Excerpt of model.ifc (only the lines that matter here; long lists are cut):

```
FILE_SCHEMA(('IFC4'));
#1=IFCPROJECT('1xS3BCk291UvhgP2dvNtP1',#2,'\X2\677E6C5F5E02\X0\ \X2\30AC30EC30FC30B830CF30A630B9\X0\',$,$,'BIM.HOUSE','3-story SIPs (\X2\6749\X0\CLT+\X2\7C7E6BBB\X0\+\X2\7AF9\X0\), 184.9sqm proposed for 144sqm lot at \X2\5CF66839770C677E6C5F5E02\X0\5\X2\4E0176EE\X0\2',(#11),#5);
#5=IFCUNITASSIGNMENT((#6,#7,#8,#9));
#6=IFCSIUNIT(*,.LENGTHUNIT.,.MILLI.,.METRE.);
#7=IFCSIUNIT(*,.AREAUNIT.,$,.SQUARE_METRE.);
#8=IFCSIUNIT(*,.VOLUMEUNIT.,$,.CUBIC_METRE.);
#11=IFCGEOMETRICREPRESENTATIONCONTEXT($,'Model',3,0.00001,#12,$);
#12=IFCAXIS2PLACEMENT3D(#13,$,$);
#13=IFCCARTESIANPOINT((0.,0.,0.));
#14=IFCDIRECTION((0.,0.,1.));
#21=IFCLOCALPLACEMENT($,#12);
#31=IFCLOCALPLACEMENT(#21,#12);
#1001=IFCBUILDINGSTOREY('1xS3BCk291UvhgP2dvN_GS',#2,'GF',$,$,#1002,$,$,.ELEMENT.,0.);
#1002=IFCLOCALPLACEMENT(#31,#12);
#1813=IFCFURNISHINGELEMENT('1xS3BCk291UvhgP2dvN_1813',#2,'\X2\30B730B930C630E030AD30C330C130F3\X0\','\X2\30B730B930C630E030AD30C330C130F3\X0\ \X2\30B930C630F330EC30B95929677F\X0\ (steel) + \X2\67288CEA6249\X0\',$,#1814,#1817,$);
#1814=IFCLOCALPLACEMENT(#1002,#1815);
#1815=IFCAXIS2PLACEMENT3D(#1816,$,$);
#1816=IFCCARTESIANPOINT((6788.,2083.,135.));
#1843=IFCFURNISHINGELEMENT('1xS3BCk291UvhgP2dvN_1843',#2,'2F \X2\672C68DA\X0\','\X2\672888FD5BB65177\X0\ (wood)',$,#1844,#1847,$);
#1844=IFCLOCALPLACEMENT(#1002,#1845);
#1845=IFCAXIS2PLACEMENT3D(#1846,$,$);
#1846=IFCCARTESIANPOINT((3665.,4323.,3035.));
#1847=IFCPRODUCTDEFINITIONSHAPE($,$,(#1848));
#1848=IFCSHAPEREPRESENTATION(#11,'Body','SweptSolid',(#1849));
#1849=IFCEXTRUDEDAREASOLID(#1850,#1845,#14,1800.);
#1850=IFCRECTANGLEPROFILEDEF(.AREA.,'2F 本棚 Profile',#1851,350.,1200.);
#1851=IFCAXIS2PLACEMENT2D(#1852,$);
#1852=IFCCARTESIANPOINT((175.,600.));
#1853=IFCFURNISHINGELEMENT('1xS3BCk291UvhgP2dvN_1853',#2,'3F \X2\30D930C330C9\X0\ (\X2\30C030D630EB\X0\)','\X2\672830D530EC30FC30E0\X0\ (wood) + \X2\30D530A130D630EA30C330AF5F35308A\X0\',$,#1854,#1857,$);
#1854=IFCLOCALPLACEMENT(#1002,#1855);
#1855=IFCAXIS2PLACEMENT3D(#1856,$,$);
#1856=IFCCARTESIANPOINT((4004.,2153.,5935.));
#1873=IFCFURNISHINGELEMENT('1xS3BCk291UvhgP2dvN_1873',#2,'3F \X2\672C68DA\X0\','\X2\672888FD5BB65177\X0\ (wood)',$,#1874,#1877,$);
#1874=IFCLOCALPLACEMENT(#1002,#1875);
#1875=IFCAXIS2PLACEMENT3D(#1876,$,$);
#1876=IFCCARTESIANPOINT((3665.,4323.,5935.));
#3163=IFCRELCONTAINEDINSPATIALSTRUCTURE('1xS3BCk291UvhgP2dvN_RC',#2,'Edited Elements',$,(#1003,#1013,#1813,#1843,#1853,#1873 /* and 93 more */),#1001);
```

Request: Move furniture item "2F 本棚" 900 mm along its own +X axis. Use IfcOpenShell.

```python
import ifcopenshell
import ifcopenshell.api.geometry
import ifcopenshell.util.placement

model = ifcopenshell.open("model.ifc")

item = model.by_guid("1xS3BCk291UvhgP2dvN_1843")
matrix = ifcopenshell.util.placement.get_local_placement(item.ObjectPlacement)
matrix[:3, 3] += matrix[:3, 0] * 900.0
ifcopenshell.api.geometry.edit_object_placement(model, product=item, matrix=matrix, is_si=False)

print(ifcopenshell.util.placement.get_local_placement(item.ObjectPlacement).round(3) + 0.0)

model.write("model_rev.ifc")
```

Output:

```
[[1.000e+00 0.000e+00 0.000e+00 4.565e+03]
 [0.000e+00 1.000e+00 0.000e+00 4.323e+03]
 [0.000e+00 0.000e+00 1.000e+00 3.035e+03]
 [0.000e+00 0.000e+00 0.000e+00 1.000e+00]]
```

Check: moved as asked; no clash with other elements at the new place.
